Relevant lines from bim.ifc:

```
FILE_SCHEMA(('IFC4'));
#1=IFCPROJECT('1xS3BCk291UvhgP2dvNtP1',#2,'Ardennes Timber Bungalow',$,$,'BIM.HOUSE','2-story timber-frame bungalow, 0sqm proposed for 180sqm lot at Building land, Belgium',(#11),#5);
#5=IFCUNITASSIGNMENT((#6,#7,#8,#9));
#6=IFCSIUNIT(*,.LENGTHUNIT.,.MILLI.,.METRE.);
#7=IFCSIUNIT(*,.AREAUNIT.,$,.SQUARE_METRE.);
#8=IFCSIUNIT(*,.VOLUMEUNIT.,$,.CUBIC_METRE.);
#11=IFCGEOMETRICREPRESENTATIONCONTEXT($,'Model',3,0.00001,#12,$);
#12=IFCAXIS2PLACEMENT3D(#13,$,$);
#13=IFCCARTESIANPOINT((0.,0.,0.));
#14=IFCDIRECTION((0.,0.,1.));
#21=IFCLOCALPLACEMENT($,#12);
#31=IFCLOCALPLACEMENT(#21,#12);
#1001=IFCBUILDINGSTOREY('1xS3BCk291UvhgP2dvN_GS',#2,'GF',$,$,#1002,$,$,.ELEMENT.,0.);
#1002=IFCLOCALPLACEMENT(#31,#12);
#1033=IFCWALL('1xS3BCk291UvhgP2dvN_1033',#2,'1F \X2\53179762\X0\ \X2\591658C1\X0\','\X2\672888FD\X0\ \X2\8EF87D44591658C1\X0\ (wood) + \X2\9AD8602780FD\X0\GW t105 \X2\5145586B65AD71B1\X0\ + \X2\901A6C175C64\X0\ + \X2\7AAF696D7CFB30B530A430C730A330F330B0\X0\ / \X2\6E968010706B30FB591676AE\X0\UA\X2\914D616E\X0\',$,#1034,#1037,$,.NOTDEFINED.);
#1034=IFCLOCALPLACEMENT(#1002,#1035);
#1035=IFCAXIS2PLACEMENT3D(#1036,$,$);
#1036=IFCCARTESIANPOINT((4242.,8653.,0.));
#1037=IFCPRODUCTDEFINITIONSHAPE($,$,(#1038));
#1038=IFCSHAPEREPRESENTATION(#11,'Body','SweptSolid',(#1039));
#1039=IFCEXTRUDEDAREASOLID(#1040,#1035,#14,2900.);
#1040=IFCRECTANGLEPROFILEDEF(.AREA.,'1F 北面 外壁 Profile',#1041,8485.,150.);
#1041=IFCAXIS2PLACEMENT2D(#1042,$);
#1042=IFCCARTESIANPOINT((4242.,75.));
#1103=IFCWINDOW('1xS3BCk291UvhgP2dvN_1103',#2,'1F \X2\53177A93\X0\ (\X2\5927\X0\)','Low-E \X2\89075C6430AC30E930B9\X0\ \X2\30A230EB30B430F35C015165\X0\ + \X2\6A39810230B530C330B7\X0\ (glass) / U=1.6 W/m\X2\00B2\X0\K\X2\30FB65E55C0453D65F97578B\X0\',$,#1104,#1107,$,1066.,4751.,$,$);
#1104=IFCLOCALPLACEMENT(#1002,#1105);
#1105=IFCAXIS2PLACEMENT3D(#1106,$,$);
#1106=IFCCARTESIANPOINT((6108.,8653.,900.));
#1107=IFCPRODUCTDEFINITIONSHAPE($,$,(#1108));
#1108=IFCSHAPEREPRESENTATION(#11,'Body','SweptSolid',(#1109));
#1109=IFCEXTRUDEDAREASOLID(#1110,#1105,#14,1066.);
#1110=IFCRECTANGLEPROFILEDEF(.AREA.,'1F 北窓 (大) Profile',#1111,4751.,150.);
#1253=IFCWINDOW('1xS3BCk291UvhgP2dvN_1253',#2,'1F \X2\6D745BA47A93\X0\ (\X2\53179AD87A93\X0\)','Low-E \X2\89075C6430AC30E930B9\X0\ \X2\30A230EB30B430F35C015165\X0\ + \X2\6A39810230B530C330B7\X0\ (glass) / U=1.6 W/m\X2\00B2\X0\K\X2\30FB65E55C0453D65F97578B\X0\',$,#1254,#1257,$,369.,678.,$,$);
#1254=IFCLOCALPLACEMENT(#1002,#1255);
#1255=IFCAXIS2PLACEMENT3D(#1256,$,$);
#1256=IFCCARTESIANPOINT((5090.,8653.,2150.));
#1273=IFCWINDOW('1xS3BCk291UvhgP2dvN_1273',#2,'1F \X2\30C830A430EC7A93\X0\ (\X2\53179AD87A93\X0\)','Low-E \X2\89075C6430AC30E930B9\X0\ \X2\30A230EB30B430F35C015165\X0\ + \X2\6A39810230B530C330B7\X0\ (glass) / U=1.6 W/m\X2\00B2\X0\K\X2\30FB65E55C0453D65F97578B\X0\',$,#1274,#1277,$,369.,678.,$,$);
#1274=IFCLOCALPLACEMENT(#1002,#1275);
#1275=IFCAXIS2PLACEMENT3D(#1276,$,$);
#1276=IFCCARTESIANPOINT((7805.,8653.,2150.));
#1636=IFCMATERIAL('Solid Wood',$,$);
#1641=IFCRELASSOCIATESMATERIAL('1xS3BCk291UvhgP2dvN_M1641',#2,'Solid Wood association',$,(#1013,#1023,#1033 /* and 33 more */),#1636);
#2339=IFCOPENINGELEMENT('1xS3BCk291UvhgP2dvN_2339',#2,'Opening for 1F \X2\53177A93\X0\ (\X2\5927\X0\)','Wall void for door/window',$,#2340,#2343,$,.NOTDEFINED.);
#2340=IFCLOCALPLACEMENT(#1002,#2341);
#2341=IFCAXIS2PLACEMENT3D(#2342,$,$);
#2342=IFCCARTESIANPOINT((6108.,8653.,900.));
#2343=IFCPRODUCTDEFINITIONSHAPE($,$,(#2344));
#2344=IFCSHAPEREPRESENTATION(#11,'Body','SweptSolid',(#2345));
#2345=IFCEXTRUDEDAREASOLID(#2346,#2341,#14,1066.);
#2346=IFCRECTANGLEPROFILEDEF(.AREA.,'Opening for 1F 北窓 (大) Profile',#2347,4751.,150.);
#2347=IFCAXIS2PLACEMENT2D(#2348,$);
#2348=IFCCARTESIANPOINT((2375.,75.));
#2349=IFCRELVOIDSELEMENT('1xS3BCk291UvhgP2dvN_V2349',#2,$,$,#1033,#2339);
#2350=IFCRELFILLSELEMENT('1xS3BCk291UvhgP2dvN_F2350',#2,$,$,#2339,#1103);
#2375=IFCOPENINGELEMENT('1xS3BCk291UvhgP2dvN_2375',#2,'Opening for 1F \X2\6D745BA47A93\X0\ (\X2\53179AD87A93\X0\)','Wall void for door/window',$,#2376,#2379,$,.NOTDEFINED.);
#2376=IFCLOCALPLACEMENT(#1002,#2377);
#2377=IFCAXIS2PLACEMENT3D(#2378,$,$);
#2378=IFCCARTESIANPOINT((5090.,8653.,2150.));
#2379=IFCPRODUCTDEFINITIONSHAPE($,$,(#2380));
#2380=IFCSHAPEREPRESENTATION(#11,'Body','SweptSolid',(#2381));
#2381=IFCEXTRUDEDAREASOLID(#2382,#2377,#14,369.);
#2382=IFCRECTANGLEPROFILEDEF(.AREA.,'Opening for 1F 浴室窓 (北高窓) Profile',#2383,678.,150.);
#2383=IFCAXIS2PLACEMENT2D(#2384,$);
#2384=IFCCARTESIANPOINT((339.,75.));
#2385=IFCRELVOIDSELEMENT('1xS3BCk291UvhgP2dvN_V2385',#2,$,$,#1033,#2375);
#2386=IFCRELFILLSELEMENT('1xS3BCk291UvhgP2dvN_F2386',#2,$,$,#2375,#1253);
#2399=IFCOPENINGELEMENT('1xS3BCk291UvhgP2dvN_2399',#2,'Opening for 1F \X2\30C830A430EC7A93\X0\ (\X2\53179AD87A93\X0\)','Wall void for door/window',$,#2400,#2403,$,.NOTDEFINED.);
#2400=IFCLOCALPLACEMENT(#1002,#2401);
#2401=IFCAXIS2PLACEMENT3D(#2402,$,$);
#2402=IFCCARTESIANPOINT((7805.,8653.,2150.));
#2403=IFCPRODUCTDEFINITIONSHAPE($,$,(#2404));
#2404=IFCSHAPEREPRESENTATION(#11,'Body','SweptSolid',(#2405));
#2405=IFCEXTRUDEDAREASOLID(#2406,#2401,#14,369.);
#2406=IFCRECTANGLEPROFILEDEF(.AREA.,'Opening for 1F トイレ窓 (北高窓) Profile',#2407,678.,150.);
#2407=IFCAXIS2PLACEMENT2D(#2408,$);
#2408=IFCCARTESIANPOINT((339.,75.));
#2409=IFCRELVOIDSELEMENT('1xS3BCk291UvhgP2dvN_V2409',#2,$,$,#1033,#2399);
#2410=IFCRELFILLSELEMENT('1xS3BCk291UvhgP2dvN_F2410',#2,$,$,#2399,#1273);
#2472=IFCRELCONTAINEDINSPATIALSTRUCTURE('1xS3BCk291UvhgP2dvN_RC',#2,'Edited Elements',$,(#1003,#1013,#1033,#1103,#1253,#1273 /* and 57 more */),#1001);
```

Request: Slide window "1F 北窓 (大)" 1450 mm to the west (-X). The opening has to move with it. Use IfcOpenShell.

```python
import ifcopenshell
import ifcopenshell.api.geometry
import ifcopenshell.util.placement

model = ifcopenshell.open("bim.ifc")

window = model.by_id(1103)
opening = window.FillsVoids[0].RelatingOpeningElement
wall = opening.VoidsElements[0].RelatingBuildingElement

wall_matrix = ifcopenshell.util.placement.get_local_placement(wall.ObjectPlacement)
shift = wall_matrix[:3, 0] * -1450.0
before = ifcopenshell.util.placement.get_local_placement(window.ObjectPlacement)[:3, 3].copy()

# The window is not placed relative to its opening, so move both.
for product in (opening, window):
    matrix = ifcopenshell.util.placement.get_local_placement(product.ObjectPlacement)
    matrix[:3, 3] += shift
    ifcopenshell.api.geometry.edit_object_placement(model, product=product, matrix=matrix, is_si=False)

after = ifcopenshell.util.placement.get_local_placement(window.ObjectPlacement)[:3, 3]
print("window moved by", (after - before).round(3) + 0.0)

model.write("bim_rev.ifc")
```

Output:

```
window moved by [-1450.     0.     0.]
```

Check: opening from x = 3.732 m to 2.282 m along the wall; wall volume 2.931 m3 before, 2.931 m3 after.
